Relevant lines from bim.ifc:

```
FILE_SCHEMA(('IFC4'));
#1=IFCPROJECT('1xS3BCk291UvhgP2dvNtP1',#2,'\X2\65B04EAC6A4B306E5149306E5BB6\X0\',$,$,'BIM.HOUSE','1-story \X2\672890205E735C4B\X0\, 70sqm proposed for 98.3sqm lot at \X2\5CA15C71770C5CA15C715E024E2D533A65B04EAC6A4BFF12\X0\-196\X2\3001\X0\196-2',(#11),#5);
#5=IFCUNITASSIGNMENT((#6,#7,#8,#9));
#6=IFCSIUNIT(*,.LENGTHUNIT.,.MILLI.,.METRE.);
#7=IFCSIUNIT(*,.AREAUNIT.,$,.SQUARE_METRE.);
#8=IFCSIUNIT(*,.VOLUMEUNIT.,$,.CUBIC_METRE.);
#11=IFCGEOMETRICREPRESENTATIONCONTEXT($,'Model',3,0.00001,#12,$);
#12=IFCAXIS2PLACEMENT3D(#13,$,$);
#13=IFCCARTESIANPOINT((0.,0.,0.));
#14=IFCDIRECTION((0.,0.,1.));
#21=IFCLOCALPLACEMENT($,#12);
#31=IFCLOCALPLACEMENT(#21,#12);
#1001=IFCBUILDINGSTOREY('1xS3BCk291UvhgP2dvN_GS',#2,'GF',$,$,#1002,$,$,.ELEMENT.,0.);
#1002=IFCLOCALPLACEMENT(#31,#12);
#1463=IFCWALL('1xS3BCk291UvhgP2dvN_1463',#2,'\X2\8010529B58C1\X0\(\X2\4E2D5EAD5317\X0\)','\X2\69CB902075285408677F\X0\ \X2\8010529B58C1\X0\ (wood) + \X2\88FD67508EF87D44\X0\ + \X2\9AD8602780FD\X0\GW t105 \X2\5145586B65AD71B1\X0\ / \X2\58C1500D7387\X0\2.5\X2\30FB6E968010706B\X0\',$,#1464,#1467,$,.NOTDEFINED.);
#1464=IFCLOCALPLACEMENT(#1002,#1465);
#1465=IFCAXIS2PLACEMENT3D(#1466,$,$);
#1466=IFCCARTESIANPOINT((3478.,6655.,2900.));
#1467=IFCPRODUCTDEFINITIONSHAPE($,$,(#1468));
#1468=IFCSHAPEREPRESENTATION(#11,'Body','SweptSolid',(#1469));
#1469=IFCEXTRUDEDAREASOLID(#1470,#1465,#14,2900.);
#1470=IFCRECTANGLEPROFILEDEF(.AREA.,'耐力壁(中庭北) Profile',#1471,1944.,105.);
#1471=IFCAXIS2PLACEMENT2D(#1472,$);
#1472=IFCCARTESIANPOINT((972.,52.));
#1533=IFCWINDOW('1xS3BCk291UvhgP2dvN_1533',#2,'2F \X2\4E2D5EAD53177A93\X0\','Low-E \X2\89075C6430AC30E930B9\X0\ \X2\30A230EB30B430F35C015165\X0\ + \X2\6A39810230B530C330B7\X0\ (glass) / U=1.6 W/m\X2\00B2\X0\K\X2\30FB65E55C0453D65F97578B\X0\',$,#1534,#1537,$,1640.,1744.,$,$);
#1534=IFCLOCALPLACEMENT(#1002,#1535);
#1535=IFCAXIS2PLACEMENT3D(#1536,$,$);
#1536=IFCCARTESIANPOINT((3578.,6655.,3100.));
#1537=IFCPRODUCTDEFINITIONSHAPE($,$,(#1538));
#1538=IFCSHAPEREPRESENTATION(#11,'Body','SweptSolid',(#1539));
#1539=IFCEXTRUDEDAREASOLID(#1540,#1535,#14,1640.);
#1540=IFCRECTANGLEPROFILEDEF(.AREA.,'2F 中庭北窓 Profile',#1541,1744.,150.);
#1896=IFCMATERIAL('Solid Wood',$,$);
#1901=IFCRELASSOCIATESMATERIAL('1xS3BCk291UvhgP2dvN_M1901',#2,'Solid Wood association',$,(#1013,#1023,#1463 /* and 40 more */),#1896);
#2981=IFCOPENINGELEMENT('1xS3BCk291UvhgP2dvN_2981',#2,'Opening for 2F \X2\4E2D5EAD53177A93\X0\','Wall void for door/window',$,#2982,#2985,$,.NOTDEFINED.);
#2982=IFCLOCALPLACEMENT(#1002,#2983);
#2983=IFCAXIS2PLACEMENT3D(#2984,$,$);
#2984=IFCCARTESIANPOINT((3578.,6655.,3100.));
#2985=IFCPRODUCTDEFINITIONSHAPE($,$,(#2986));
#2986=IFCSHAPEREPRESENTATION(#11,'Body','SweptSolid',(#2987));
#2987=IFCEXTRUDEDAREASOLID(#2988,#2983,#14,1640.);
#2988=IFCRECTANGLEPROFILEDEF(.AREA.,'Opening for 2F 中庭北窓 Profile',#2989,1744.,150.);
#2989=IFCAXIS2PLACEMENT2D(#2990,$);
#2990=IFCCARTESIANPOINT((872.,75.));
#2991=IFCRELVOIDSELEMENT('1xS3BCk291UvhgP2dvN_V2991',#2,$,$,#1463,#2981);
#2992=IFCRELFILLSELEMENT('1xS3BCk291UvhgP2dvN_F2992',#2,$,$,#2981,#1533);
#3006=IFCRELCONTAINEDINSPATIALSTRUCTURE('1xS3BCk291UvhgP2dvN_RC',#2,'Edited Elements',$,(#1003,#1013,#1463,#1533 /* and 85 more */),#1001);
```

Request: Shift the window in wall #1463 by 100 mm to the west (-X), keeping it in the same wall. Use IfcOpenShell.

```python
import ifcopenshell
import ifcopenshell.api.geometry
import ifcopenshell.util.placement

model = ifcopenshell.open("bim.ifc")

window = model.by_guid("1xS3BCk291UvhgP2dvN_1533")
opening = window.FillsVoids[0].RelatingOpeningElement
wall = opening.VoidsElements[0].RelatingBuildingElement

wall_matrix = ifcopenshell.util.placement.get_local_placement(wall.ObjectPlacement)
shift = wall_matrix[:3, 0] * -100.0
before = ifcopenshell.util.placement.get_local_placement(window.ObjectPlacement)[:3, 3].copy()

# The window is not placed relative to its opening, so move both.
for product in (opening, window):
    matrix = ifcopenshell.util.placement.get_local_placement(product.ObjectPlacement)
    matrix[:3, 3] += shift
    ifcopenshell.api.geometry.edit_object_placement(model, product=product, matrix=matrix, is_si=False)

after = ifcopenshell.util.placement.get_local_placement(window.ObjectPlacement)[:3, 3]
print("window moved by", (after - before).round(3) + 0.0)

model.write("bim_updated.ifc")
```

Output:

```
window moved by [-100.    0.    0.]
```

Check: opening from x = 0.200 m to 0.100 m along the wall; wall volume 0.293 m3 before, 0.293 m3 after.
